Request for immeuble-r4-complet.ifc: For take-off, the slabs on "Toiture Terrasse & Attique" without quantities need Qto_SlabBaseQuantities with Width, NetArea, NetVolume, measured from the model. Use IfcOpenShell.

First a look at what the model holds.

```python
import ifcopenshell
import ifcopenshell.util.element
import ifcopenshell.util.unit

model = ifcopenshell.open("immeuble-r4-complet.ifc")
print(model.schema)
for unit_type in ("LENGTHUNIT", "AREAUNIT", "VOLUMEUNIT"):
    print(unit_type, ifcopenshell.util.unit.calculate_unit_scale(model, unit_type))
storey = next(s for s in model.by_type("IfcBuildingStorey") if s.Name == "Toiture Terrasse & Attique")
slabs = [e for e in ifcopenshell.util.element.get_decomposition(storey) if e.is_a("IfcSlab")]
for e in sorted(slabs, key=lambda e: e.id()):
    print(e.id(), e.is_a(), e.Name, list(ifcopenshell.util.element.get_psets(e, qtos_only=True)), sep=" | ")
```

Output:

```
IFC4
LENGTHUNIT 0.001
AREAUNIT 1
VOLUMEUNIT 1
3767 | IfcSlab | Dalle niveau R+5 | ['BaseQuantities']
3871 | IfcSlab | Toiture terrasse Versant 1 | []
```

```python
import ifcopenshell
import ifcopenshell.api.pset
import ifcopenshell.geom
import ifcopenshell.util.element
import ifcopenshell.util.shape
import ifcopenshell.util.unit

model = ifcopenshell.open("immeuble-r4-complet.ifc")
unit_scale = ifcopenshell.util.unit.calculate_unit_scale(model)
area_scale = ifcopenshell.util.unit.calculate_unit_scale(model, "AREAUNIT")
volume_scale = ifcopenshell.util.unit.calculate_unit_scale(model, "VOLUMEUNIT")
settings = ifcopenshell.geom.settings()

storey = next(s for s in model.by_type("IfcBuildingStorey") if s.Name == "Toiture Terrasse & Attique")
slabs = [e for e in ifcopenshell.util.element.get_decomposition(storey) if e.is_a("IfcSlab")]

for e in sorted(slabs, key=lambda e: e.id()):
    if ifcopenshell.util.element.get_psets(e, qtos_only=True, should_inherit=False):
        continue
    # Geometry comes back in metres, in the element's own axes.
    shape = ifcopenshell.geom.create_shape(settings, e)
    values = {
        "Width": ifcopenshell.util.shape.get_z(shape.geometry) / unit_scale,
        "NetArea": ifcopenshell.util.shape.get_footprint_area(shape.geometry) / area_scale,
        "NetVolume": ifcopenshell.util.shape.get_volume(shape.geometry) / volume_scale,
    }
    qto = ifcopenshell.api.pset.add_qto(model, product=e, name="Qto_SlabBaseQuantities")
    ifcopenshell.api.pset.edit_qto(model, qto=qto, properties=values)
    print(e.id(), {k: round(v, 3) for k, v in values.items()})

model.write("immeuble-r4-complet_updated.ifc")
```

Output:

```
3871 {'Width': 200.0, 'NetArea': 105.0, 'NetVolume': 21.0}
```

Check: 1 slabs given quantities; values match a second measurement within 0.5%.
